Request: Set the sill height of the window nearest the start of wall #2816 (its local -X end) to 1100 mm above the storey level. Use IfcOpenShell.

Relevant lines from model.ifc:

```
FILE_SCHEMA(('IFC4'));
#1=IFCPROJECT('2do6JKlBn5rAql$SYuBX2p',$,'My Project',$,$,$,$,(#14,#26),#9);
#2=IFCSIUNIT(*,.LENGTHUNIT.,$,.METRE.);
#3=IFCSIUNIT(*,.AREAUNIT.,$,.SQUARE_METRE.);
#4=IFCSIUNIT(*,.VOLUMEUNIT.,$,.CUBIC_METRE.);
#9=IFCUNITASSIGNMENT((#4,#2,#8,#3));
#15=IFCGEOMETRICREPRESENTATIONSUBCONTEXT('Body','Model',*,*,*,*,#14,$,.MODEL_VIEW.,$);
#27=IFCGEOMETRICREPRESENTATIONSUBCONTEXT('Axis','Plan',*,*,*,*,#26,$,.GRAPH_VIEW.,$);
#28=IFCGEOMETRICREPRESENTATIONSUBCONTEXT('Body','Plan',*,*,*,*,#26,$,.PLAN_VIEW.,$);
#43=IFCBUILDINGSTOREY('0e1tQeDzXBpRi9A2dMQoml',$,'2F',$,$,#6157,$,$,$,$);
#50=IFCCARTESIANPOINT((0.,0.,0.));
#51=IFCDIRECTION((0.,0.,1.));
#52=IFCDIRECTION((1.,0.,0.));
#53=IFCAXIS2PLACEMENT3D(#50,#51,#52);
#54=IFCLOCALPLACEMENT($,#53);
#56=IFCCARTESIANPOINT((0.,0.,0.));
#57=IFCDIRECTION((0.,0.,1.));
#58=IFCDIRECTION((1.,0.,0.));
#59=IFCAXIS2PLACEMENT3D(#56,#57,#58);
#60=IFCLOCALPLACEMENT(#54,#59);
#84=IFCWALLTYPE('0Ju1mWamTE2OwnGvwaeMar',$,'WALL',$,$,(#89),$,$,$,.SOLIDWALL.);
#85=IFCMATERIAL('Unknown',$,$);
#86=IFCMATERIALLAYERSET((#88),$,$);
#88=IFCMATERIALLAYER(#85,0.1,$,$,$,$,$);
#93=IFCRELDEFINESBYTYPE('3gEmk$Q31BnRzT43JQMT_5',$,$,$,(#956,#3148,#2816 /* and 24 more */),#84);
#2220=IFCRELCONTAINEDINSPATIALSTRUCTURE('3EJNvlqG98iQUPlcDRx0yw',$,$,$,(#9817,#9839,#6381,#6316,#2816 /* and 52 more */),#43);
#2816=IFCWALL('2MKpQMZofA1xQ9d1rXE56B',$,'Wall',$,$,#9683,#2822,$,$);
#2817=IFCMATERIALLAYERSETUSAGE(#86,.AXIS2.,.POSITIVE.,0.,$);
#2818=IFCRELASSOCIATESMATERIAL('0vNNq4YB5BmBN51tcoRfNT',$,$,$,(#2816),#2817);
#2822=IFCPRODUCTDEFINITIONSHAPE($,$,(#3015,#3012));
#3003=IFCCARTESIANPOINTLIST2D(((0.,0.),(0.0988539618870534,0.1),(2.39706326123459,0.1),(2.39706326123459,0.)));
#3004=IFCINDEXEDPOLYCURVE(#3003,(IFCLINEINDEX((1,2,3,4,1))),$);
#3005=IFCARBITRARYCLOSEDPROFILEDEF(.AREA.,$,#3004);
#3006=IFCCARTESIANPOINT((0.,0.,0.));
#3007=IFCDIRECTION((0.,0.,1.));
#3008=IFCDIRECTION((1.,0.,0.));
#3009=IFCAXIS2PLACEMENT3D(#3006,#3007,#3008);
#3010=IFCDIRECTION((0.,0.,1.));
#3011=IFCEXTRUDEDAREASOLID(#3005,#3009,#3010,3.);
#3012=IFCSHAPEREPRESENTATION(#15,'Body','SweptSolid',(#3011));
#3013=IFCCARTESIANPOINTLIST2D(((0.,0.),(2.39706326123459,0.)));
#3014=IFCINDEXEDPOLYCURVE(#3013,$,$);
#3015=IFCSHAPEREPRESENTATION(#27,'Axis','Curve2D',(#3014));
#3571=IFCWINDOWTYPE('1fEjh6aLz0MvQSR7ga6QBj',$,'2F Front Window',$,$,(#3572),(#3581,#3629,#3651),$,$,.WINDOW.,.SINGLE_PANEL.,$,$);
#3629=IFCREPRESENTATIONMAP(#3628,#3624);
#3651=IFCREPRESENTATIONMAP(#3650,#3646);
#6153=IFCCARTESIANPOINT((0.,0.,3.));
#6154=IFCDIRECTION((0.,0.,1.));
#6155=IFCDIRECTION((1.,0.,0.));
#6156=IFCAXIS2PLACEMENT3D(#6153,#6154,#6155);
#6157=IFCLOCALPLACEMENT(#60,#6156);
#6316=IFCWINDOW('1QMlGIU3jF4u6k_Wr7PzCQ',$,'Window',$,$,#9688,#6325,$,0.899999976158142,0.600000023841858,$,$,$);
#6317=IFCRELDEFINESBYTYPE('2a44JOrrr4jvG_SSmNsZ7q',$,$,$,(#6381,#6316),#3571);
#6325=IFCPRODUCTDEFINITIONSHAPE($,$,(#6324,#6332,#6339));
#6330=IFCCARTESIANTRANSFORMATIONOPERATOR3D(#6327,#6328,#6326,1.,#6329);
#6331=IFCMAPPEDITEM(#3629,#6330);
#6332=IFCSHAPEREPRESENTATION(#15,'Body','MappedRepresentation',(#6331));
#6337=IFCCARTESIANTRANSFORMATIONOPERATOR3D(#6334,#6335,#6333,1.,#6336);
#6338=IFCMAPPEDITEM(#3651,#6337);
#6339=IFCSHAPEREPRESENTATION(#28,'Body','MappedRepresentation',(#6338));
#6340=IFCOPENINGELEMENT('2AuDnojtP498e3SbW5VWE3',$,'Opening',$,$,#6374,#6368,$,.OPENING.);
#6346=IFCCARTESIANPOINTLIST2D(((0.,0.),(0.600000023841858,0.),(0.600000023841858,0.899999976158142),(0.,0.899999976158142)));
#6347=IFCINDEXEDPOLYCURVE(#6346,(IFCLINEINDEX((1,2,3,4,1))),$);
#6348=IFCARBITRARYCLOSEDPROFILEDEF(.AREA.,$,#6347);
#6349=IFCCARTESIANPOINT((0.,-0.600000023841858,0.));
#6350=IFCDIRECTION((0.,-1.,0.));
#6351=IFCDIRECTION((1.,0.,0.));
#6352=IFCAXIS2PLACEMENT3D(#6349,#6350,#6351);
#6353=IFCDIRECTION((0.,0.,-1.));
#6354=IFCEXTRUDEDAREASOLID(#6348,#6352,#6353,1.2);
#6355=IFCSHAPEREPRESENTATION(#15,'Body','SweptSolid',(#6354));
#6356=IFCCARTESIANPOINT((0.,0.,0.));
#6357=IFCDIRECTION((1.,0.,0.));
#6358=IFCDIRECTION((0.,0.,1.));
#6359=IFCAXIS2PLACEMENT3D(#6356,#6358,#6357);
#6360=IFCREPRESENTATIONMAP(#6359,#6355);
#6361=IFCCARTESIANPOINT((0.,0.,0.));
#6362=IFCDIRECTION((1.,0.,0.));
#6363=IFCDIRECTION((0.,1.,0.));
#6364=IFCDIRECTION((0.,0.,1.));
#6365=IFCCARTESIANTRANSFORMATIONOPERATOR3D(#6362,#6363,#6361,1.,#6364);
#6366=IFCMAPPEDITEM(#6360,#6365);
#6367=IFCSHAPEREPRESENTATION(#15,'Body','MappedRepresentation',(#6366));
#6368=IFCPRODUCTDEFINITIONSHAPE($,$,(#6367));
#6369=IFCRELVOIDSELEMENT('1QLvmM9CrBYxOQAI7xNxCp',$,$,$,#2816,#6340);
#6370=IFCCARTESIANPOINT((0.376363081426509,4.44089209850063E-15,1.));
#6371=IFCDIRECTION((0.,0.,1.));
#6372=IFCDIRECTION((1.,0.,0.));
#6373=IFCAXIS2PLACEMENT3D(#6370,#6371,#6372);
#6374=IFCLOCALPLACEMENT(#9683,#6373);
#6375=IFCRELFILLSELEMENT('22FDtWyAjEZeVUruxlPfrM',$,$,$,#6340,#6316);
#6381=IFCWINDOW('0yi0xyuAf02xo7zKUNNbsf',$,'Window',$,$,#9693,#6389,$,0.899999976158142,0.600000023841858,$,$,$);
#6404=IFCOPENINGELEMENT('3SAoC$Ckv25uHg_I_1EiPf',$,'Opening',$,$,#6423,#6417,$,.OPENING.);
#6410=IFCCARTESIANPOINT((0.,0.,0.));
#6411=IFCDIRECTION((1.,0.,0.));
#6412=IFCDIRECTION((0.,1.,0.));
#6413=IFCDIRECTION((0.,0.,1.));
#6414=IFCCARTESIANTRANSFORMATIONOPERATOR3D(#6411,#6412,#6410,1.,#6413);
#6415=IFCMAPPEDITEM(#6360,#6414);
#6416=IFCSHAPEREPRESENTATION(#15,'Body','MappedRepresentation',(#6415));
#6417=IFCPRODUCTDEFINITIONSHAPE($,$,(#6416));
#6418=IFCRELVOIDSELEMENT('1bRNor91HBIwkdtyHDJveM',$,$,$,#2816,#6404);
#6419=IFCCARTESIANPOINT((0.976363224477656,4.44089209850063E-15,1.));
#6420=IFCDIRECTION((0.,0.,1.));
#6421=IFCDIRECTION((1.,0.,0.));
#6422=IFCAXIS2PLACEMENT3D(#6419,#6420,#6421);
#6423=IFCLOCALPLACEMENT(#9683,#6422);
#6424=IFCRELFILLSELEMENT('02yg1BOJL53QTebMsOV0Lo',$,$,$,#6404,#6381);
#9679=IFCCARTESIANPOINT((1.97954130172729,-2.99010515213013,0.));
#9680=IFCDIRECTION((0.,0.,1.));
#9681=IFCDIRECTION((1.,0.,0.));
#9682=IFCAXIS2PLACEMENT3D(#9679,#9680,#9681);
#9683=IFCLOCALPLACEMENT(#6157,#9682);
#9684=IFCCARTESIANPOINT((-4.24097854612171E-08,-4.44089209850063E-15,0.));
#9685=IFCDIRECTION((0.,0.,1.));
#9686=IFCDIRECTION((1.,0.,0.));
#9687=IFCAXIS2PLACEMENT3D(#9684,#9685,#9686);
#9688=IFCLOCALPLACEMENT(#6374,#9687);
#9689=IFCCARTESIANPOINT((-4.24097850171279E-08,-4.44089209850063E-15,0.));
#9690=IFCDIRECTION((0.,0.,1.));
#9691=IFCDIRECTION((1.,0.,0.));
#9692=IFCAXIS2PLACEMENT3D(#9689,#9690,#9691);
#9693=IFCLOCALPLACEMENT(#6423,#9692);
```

```python
import numpy as np
import ifcopenshell
import ifcopenshell.api.geometry
import ifcopenshell.geom
import ifcopenshell.util.element
import ifcopenshell.util.placement
import ifcopenshell.util.shape
import ifcopenshell.util.unit

model = ifcopenshell.open("model.ifc")
unit_scale = ifcopenshell.util.unit.calculate_unit_scale(model)

window = model.by_guid("1QMlGIU3jF4u6k_Wr7PzCQ")
opening = window.FillsVoids[0].RelatingOpeningElement
storey = ifcopenshell.util.element.get_container(window, ifc_class="IfcBuildingStorey")
level = ifcopenshell.util.placement.get_local_placement(storey.ObjectPlacement)[2, 3]

# The opening's origin need not be at the sill, so measure its lowest point.
shape = ifcopenshell.geom.create_shape(ifcopenshell.geom.settings(), opening)
bottom = ifcopenshell.util.shape.get_shape_bottom_elevation(shape, shape.geometry) / unit_scale
dz = level + 1.1 / unit_scale - bottom

shift = np.array([0.0, 0.0, dz])
# The window is placed relative to its opening, so it follows when the opening moves.
matrix = ifcopenshell.util.placement.get_local_placement(opening.ObjectPlacement)
matrix[:3, 3] += shift
ifcopenshell.api.geometry.edit_object_placement(
    model, product=opening, matrix=matrix, is_si=False, should_transform_children=True
)

print(f"moved by {dz * unit_scale:+.3f} m")

model.write("model_v2.ifc")
```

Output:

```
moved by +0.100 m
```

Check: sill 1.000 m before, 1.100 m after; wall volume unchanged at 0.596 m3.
